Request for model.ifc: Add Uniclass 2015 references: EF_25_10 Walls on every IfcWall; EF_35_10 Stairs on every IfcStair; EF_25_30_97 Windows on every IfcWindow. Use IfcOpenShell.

First a look at what the model holds.

```python
import ifcopenshell

model = ifcopenshell.open("model.ifc")
print(model.schema)
print("classifications:", [c.Name for c in model.by_type("IfcClassification")])
for ifc_class in ("IfcDoor", "IfcRoof", "IfcStair", "IfcWall", "IfcWindow"):
    print(ifc_class, len(model.by_type(ifc_class)))
```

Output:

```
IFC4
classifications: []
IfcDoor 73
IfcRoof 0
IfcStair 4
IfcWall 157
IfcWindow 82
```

```python
import ifcopenshell
import ifcopenshell.api.classification

model = ifcopenshell.open("model.ifc")

system = ifcopenshell.api.classification.add_classification(model, classification="Uniclass 2015")

codes = {
    "IfcWall": ("EF_25_10", "Walls"),
    "IfcStair": ("EF_35_10", "Stairs"),
    "IfcWindow": ("EF_25_30_97", "Windows"),
}
for ifc_class, (code, name) in codes.items():
    products = model.by_type(ifc_class)
    ifcopenshell.api.classification.add_reference(
        model, products=products, classification=system, identification=code, name=name
    )
    print(code, len(products))

model.write("model_rev.ifc")
```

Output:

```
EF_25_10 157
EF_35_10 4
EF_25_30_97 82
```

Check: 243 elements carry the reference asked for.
